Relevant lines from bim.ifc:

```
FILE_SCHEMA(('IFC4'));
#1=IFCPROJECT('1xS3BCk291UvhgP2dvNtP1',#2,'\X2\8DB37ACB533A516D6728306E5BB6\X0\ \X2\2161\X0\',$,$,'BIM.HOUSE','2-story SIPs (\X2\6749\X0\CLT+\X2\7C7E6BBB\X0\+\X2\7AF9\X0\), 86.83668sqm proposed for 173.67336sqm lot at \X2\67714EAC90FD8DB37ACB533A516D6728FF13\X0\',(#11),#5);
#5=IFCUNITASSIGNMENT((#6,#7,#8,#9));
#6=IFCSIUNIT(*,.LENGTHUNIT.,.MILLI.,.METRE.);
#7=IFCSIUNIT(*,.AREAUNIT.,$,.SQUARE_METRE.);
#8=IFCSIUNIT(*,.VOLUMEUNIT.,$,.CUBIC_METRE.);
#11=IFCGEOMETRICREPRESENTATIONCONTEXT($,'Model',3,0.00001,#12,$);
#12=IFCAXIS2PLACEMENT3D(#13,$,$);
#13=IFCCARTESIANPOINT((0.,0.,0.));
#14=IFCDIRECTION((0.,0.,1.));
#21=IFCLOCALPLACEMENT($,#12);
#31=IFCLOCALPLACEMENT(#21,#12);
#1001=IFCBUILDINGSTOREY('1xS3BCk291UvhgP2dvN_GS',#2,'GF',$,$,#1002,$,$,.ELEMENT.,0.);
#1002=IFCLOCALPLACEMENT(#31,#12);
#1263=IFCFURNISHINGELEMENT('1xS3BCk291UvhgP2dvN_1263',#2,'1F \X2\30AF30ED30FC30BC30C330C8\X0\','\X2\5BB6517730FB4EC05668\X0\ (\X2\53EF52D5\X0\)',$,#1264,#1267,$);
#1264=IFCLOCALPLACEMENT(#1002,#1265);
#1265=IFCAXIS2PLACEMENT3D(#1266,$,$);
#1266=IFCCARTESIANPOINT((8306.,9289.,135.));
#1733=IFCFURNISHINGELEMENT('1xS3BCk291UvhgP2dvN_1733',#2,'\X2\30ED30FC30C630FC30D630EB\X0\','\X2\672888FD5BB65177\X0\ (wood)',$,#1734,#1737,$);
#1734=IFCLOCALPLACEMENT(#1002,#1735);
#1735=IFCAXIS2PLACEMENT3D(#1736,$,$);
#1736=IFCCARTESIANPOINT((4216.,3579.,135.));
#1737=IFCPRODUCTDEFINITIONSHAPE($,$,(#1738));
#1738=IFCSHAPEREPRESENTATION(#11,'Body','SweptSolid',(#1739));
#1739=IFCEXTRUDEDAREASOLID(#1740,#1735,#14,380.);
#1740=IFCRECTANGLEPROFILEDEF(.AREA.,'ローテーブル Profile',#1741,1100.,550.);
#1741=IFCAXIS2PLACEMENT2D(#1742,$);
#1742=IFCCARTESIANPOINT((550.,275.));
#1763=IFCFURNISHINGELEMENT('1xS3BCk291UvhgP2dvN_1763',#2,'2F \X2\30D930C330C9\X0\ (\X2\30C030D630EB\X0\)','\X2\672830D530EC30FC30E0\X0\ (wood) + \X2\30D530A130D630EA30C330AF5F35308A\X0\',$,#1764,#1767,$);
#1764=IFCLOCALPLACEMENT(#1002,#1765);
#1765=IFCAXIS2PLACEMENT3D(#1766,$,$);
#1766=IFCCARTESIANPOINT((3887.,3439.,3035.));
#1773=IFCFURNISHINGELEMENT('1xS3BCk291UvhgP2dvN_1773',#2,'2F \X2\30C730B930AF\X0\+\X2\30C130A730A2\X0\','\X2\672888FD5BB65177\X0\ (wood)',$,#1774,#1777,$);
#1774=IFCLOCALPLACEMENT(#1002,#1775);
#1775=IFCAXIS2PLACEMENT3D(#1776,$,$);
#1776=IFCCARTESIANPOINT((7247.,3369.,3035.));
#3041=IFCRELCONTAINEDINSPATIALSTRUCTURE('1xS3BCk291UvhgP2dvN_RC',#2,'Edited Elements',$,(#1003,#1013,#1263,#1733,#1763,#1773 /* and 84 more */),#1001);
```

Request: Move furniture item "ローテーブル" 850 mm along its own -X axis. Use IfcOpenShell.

```python
import ifcopenshell
import ifcopenshell.api.geometry
import ifcopenshell.util.placement
import ifcopenshell.util.unit

model = ifcopenshell.open("bim.ifc")
unit_scale = ifcopenshell.util.unit.calculate_unit_scale(model)

item = model.by_guid("1xS3BCk291UvhgP2dvN_1733")
matrix = ifcopenshell.util.placement.get_local_placement(item.ObjectPlacement)
matrix[:3, 3] -= matrix[:3, 0] * 0.85 / unit_scale
ifcopenshell.api.geometry.edit_object_placement(model, product=item, matrix=matrix, is_si=False)

print(ifcopenshell.util.placement.get_local_placement(item.ObjectPlacement).round(3) + 0.0)

model.write("bim-out.ifc")
```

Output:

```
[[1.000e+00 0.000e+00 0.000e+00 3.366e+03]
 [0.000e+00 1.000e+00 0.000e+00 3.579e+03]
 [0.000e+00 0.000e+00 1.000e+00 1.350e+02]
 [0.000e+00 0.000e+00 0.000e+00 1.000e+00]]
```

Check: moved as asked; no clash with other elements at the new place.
